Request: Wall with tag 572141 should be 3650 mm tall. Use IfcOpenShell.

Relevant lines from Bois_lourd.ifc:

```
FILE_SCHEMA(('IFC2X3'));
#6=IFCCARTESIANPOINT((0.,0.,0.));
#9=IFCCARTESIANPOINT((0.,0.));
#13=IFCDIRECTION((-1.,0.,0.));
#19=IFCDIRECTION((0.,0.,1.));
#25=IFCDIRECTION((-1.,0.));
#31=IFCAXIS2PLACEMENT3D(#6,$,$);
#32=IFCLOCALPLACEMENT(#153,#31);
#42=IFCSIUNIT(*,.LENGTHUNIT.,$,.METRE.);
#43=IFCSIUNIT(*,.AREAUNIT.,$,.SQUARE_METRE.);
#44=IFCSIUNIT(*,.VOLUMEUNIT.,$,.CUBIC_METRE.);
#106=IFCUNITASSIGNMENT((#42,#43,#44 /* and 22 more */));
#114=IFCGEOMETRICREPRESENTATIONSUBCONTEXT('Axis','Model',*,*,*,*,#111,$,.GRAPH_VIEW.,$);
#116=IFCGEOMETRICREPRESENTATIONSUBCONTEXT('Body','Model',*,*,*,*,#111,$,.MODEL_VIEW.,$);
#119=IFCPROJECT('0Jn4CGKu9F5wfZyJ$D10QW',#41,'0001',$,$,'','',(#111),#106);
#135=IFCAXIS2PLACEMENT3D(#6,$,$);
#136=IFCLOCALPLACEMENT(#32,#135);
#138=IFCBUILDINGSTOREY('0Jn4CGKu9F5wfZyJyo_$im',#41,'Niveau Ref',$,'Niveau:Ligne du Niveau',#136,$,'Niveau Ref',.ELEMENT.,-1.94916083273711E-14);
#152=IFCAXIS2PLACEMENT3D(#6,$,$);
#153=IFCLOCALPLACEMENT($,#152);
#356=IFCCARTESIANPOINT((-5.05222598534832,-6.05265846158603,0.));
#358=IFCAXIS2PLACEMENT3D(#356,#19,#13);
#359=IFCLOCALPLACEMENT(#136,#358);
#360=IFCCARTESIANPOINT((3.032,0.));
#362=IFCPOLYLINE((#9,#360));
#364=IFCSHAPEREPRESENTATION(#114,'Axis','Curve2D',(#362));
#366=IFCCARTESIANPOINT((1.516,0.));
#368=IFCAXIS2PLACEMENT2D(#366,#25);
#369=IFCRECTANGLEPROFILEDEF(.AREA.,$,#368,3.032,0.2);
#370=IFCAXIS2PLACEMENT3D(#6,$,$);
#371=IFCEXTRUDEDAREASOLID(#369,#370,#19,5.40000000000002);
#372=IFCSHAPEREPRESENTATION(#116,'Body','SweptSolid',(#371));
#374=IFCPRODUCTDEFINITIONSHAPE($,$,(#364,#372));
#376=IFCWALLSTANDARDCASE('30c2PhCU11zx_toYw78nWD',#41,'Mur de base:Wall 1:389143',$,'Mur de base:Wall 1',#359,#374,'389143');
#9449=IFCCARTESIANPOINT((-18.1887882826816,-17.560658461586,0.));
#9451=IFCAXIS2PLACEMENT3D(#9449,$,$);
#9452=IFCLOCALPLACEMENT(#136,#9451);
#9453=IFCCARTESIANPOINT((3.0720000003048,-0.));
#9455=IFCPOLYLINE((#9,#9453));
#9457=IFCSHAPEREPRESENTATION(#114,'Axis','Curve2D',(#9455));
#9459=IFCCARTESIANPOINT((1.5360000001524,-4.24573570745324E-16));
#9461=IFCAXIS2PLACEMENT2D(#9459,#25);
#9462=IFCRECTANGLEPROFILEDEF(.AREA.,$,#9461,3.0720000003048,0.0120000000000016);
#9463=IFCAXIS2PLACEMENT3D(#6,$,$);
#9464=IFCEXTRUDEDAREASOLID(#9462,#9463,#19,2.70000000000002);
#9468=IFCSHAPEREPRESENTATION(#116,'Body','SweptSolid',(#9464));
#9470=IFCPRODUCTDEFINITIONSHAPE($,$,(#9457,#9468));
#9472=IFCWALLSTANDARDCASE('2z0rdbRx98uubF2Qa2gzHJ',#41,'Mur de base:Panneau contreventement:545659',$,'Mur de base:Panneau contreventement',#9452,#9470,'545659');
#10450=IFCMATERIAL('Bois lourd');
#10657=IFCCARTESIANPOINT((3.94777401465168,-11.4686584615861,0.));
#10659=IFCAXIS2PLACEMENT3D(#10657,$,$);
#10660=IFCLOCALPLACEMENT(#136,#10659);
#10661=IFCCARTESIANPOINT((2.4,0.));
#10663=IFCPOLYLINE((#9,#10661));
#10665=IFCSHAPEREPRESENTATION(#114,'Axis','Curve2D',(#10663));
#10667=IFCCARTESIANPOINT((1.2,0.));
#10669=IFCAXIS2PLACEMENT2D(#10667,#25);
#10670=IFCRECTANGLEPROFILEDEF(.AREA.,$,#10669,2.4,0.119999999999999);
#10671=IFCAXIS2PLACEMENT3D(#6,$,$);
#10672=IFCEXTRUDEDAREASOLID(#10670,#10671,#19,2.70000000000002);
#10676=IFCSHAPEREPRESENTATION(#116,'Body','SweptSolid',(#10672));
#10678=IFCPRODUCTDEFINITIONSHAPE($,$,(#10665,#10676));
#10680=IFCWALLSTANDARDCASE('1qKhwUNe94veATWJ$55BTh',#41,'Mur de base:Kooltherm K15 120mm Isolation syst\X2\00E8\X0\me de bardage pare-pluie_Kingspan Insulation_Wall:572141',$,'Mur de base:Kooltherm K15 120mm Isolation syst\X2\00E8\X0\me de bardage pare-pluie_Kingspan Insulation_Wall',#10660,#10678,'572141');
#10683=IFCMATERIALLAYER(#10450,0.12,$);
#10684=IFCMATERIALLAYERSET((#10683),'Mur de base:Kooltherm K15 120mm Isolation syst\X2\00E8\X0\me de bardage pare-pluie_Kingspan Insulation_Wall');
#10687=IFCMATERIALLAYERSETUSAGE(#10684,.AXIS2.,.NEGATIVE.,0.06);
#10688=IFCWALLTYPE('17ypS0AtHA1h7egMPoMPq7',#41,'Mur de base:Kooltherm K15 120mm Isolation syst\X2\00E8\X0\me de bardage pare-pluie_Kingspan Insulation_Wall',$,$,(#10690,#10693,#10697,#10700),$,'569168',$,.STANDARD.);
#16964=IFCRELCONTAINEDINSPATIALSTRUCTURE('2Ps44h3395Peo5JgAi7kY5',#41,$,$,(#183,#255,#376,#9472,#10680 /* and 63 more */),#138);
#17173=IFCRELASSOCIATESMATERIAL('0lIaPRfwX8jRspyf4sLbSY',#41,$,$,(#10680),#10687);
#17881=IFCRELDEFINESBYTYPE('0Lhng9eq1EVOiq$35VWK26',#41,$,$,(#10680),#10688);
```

```python
import ifcopenshell
import ifcopenshell.geom
import ifcopenshell.util.representation
import ifcopenshell.util.shape
import ifcopenshell.util.unit

model = ifcopenshell.open("Bois_lourd.ifc")
unit_scale = ifcopenshell.util.unit.calculate_unit_scale(model)
settings = ifcopenshell.geom.settings()


def volume(element):
    """Net volume in cubic metres, openings subtracted."""
    shape = ifcopenshell.geom.create_shape(settings, element)
    return ifcopenshell.util.shape.get_volume(shape.geometry)


wall = model.by_guid("1qKhwUNe94veATWJ$55BTh")
before = volume(wall)

body = ifcopenshell.util.representation.get_representation(wall, "Model", "Body")
solid = body.Items[0]
old_height = solid.Depth
solid.Depth = 3.65 / unit_scale
after = volume(wall)

print(f"height {old_height:g} -> {solid.Depth:g}, volume {before:.3f} -> {after:.3f} m3")

model.write("Bois_lourd_updated.ifc")
```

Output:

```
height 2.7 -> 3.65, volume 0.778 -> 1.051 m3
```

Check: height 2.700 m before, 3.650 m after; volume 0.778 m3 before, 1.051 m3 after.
